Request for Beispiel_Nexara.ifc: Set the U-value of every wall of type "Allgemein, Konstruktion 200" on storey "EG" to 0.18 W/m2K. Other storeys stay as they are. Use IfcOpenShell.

First a look at what the model holds.

```python
import ifcopenshell
import ifcopenshell.util.element

model = ifcopenshell.open("Beispiel_Nexara.ifc")
print(model.schema)
storey = next(s for s in model.by_type("IfcBuildingStorey") if s.Name == "EG")
walls = [e for e in ifcopenshell.util.element.get_decomposition(storey) if e.is_a("IfcWall")]
seen = {}
for e in walls:
    element_type = ifcopenshell.util.element.get_type(e)
    key = (element_type.Name if element_type != e and element_type else None, ifcopenshell.util.element.get_pset(e, "Pset_WallCommon", "ThermalTransmittance"))
    seen[key] = seen.get(key, 0) + 1
for (name, value), count in sorted(seen.items(), key=str):
    print(count, "x", name, "|", value)
```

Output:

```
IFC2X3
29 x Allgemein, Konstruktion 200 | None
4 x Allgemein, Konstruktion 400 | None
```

```python
import ifcopenshell
import ifcopenshell.api.pset
import ifcopenshell.util.element

model = ifcopenshell.open("Beispiel_Nexara.ifc")

storey = next(s for s in model.by_type("IfcBuildingStorey") if s.Name == "EG")
walls = [e for e in ifcopenshell.util.element.get_decomposition(storey) if e.is_a("IfcWall")]

count = 0
for e in walls:
    element_type = ifcopenshell.util.element.get_type(e)
    if element_type in (None, e) or element_type.Name != "Allgemein, Konstruktion 200":
        continue
    # add_pset returns the element's existing set when there is one.
    pset = ifcopenshell.api.pset.add_pset(model, product=e, name="Pset_WallCommon")
    ifcopenshell.api.pset.edit_pset(model, pset=pset, properties={"ThermalTransmittance": 0.18})
    count += 1

print(count, "walls updated")

model.write("Beispiel_Nexara_edited.ifc")
```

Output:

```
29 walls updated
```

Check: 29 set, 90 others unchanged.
